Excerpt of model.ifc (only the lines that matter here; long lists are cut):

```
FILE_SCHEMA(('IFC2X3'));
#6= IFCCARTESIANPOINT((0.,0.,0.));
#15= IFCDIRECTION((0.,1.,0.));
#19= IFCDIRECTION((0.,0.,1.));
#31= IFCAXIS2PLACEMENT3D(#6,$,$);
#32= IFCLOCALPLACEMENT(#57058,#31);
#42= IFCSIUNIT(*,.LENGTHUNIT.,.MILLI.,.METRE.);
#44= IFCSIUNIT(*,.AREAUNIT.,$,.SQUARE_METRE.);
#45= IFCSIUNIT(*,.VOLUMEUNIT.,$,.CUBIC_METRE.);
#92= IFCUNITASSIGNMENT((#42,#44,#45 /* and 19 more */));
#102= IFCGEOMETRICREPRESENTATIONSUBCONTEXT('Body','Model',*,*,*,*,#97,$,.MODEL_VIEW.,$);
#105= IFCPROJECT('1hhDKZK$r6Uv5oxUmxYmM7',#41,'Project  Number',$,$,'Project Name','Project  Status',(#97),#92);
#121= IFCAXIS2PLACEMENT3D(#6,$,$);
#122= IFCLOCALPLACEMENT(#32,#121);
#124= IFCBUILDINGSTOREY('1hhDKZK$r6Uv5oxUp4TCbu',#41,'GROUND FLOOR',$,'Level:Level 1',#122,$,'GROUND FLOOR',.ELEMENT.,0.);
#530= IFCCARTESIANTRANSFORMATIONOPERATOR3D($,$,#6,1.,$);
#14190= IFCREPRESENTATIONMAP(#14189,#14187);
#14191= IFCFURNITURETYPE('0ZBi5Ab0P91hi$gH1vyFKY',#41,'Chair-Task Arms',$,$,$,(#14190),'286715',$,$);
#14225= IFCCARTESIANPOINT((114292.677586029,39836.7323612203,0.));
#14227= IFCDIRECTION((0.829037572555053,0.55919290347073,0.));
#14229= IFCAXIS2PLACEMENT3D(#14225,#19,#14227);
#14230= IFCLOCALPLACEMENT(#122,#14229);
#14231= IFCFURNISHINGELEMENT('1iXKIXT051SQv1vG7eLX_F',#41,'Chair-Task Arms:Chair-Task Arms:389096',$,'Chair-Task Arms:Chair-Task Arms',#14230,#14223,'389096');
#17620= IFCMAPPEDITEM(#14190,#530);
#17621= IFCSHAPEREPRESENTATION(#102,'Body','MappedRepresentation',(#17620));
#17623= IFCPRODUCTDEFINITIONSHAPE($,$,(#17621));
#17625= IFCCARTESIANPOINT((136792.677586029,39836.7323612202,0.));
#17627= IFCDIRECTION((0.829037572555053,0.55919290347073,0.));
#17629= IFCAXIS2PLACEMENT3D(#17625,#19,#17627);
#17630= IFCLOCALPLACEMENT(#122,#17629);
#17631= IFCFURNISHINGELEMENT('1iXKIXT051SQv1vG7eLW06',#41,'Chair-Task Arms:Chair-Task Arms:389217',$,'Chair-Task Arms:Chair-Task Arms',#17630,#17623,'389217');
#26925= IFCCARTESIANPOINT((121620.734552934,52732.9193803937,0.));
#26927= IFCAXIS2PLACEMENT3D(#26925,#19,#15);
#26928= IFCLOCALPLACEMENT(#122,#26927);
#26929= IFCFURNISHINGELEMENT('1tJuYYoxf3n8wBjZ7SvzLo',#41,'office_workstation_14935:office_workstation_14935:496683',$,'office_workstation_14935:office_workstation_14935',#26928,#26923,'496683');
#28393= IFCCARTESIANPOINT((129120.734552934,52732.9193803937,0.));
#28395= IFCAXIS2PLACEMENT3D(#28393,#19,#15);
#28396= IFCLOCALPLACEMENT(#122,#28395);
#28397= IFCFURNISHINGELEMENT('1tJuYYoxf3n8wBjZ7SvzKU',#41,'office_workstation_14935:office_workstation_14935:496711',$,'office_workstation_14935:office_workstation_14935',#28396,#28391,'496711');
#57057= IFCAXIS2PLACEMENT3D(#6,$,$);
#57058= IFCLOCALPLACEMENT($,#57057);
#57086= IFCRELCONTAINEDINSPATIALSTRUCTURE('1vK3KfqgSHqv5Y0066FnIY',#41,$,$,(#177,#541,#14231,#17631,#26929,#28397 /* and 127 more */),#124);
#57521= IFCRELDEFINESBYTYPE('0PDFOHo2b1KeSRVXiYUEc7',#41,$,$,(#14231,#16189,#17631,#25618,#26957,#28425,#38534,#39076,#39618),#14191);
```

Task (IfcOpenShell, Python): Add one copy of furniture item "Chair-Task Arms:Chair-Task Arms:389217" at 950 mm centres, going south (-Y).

```python
import numpy as np
import ifcopenshell
import ifcopenshell.api.geometry
import ifcopenshell.api.root
import ifcopenshell.util.element
import ifcopenshell.util.placement
import ifcopenshell.util.unit

model = ifcopenshell.open("model.ifc")
unit_scale = ifcopenshell.util.unit.calculate_unit_scale(model)


def reuse_history(source, copy):
    """copy_class also copies each property set's owner history, people and application; keep the originals."""
    for rel in copy.IsDefinedBy:
        if rel.is_a("IfcRelDefinesByProperties") and (history := rel.RelatingPropertyDefinition.OwnerHistory):
            rel.RelatingPropertyDefinition.OwnerHistory = source.OwnerHistory
            ifcopenshell.util.element.remove_deep2(model, history)


source = model.by_id(17631)
base = ifcopenshell.util.placement.get_local_placement(source.ObjectPlacement)
step = np.array([0.0, -1.0, 0.0]) * 0.95 / unit_scale

for i in range(1, 2):
    copy = ifcopenshell.api.root.copy_class(model, product=source)
    copy.Representation = ifcopenshell.util.element.copy_deep(
        model, source.Representation, exclude=["IfcGeometricRepresentationContext", "IfcRepresentationMap"]
    )
    copy.Name = "Chair-Task Arms:Chair-Task Arms"
    copy.Tag = None
    reuse_history(source, copy)
    matrix = base.copy()
    matrix[:3, 3] += i * step
    print("added at", matrix[:3, 3].round(3) + 0.0)
    ifcopenshell.api.geometry.edit_object_placement(model, product=copy, matrix=matrix, is_si=False)

model.write("model_edited.ifc")
```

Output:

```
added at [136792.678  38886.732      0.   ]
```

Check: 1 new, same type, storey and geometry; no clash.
